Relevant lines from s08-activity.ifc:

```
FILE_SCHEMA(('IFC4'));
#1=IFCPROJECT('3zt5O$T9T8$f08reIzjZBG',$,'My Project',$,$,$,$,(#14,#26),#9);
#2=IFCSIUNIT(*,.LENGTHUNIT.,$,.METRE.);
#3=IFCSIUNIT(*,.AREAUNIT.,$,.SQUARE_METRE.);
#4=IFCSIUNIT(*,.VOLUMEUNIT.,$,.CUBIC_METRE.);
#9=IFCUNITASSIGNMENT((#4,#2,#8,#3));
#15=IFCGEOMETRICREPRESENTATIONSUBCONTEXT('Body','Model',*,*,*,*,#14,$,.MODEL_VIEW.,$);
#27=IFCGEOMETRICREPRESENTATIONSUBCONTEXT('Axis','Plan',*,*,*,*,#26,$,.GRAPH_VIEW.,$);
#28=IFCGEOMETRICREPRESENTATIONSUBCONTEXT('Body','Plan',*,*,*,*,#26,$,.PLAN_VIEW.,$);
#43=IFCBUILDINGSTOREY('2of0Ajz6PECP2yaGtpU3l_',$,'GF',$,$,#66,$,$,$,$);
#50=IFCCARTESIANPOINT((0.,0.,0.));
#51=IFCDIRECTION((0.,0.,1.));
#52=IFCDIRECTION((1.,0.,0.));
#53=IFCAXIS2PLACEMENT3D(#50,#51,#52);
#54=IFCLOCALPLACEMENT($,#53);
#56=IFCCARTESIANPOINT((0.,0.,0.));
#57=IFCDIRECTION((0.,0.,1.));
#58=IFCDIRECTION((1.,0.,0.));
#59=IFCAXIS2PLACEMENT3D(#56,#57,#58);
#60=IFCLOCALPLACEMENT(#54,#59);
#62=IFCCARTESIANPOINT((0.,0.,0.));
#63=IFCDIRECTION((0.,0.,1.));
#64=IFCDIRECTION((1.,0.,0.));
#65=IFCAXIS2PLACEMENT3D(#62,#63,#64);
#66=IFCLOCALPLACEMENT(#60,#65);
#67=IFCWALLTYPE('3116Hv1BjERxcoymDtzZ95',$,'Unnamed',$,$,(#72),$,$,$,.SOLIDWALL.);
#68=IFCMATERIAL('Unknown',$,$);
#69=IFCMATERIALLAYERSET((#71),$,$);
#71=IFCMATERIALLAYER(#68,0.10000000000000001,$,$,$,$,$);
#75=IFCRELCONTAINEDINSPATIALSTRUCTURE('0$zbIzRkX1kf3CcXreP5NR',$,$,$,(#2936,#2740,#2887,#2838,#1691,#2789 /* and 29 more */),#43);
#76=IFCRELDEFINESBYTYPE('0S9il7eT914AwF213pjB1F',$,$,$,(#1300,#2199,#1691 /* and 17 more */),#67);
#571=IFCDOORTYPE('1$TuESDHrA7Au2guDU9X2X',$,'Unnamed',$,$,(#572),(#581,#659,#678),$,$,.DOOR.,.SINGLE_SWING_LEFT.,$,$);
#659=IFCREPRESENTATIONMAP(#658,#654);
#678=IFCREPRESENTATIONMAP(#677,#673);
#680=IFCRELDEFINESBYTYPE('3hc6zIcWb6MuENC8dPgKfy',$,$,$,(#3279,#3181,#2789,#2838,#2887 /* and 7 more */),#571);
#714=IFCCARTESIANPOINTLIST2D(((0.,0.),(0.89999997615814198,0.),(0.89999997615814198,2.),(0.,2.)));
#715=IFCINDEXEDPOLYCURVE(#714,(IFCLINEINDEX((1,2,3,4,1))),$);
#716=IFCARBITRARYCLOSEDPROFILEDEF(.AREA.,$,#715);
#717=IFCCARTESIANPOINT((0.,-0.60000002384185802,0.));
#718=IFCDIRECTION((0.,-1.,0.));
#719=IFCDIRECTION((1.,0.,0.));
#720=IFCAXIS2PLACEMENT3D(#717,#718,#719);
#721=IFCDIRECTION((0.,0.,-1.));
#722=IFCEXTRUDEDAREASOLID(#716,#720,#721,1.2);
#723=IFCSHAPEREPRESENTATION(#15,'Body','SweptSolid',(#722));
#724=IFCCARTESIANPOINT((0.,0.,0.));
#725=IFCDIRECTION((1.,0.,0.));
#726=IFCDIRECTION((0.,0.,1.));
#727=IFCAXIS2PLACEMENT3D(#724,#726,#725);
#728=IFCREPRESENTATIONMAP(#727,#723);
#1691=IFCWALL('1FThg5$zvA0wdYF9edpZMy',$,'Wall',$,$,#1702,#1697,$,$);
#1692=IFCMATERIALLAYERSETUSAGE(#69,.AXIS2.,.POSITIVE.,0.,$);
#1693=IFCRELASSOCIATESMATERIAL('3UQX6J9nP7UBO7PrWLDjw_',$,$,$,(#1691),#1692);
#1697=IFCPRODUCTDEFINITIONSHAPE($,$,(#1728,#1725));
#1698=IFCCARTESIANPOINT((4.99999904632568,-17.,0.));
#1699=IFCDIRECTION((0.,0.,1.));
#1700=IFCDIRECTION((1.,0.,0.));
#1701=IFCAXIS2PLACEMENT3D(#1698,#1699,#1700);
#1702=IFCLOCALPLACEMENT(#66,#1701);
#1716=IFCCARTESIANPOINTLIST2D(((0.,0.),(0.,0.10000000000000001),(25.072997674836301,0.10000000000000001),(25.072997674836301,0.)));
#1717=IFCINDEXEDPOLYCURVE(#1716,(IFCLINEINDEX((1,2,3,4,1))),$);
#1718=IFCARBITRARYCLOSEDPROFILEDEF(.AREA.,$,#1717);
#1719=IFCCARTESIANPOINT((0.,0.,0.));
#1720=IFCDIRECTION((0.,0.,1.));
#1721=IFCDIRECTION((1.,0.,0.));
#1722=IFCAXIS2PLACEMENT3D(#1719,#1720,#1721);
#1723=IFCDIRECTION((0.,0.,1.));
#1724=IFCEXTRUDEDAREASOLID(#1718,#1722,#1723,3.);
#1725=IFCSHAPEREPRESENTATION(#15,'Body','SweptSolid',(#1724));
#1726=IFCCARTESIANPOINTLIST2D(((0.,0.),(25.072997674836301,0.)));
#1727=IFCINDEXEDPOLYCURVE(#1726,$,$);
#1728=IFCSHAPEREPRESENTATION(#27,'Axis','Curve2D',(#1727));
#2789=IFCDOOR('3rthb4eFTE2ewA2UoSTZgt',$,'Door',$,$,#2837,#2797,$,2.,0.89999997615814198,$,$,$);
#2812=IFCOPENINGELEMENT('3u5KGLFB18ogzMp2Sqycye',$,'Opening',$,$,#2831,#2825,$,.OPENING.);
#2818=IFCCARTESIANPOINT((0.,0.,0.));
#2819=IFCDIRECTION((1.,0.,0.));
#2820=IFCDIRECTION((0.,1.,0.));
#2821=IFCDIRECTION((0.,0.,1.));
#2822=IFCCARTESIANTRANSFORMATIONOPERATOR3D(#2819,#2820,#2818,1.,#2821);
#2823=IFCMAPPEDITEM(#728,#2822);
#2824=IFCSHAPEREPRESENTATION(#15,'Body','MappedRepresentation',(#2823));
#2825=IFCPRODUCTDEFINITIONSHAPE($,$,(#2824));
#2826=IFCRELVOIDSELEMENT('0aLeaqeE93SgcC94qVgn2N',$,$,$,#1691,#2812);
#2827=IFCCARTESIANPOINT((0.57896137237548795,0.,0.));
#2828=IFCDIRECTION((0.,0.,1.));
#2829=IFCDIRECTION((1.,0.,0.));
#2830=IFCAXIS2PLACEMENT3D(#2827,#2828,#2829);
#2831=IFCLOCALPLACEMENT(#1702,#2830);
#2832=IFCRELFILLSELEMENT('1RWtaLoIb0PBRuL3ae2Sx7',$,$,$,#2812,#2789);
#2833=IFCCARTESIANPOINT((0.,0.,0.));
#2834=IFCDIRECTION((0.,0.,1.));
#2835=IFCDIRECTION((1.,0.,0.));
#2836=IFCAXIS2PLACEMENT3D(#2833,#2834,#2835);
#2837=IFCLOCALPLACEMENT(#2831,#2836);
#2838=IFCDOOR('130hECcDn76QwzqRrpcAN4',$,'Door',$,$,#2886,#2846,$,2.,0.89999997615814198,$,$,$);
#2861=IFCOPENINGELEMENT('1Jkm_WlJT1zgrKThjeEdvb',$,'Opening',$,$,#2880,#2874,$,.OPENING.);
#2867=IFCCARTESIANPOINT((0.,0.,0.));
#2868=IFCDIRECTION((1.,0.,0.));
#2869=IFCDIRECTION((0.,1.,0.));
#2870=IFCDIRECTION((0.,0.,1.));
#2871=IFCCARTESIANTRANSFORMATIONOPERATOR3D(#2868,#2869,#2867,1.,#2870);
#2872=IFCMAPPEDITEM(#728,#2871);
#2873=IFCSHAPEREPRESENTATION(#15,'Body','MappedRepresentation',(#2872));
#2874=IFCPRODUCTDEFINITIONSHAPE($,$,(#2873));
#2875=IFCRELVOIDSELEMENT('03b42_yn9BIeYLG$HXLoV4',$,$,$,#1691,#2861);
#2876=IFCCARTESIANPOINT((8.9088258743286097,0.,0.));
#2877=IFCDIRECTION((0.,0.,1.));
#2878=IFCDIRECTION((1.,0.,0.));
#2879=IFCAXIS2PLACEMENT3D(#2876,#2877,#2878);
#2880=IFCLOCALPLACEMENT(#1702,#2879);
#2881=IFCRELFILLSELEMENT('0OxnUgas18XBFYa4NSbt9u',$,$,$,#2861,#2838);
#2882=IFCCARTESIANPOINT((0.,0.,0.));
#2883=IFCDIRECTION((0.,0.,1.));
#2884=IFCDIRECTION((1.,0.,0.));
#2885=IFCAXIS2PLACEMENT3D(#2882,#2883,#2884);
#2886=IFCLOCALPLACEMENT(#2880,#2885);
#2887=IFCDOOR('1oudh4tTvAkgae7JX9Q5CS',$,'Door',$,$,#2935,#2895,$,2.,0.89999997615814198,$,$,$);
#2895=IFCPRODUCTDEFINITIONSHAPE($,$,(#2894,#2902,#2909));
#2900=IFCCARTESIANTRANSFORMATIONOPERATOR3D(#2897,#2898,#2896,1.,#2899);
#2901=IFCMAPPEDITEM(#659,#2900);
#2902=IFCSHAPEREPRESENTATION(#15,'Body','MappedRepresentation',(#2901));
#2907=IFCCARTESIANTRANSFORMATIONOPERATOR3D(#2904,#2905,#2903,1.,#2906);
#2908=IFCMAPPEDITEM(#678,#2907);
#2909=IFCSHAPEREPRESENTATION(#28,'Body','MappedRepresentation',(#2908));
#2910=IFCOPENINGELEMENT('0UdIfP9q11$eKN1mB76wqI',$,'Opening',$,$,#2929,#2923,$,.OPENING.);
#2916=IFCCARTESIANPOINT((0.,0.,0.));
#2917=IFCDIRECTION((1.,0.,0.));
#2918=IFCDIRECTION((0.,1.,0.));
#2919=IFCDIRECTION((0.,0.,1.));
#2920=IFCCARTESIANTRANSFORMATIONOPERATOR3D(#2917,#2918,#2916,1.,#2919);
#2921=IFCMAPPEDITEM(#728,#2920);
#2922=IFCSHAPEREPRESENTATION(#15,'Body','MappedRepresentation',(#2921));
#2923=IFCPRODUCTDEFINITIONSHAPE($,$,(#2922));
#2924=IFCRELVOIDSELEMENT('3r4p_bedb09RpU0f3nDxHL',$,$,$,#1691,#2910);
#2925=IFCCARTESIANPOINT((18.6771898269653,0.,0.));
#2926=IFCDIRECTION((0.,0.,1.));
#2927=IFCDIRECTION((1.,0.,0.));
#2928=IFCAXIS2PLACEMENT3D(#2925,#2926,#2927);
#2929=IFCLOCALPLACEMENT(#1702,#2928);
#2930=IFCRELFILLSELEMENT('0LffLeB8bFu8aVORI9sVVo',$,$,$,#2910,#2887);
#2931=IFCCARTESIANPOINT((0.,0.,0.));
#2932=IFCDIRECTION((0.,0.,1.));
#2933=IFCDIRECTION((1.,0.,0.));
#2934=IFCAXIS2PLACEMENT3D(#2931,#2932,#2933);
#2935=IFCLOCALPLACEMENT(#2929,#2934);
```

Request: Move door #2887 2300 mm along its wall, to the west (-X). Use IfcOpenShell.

```python
import ifcopenshell
import ifcopenshell.api.geometry
import ifcopenshell.util.placement

model = ifcopenshell.open("s08-activity.ifc")

door = model.by_guid("1oudh4tTvAkgae7JX9Q5CS")
opening = door.FillsVoids[0].RelatingOpeningElement
wall = opening.VoidsElements[0].RelatingBuildingElement

wall_matrix = ifcopenshell.util.placement.get_local_placement(wall.ObjectPlacement)
shift = wall_matrix[:3, 0] * -2.3
before = ifcopenshell.util.placement.get_local_placement(door.ObjectPlacement)[:3, 3].copy()

# The door is placed relative to its opening, so it follows when the opening moves.
matrix = ifcopenshell.util.placement.get_local_placement(opening.ObjectPlacement)
matrix[:3, 3] += shift
ifcopenshell.api.geometry.edit_object_placement(
    model, product=opening, matrix=matrix, is_si=False, should_transform_children=True
)

after = ifcopenshell.util.placement.get_local_placement(door.ObjectPlacement)[:3, 3]
print("door moved by", (after - before).round(3) + 0.0)

model.write("s08-activity_updated.ifc")
```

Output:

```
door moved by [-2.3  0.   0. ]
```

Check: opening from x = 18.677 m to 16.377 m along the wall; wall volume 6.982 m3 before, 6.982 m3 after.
